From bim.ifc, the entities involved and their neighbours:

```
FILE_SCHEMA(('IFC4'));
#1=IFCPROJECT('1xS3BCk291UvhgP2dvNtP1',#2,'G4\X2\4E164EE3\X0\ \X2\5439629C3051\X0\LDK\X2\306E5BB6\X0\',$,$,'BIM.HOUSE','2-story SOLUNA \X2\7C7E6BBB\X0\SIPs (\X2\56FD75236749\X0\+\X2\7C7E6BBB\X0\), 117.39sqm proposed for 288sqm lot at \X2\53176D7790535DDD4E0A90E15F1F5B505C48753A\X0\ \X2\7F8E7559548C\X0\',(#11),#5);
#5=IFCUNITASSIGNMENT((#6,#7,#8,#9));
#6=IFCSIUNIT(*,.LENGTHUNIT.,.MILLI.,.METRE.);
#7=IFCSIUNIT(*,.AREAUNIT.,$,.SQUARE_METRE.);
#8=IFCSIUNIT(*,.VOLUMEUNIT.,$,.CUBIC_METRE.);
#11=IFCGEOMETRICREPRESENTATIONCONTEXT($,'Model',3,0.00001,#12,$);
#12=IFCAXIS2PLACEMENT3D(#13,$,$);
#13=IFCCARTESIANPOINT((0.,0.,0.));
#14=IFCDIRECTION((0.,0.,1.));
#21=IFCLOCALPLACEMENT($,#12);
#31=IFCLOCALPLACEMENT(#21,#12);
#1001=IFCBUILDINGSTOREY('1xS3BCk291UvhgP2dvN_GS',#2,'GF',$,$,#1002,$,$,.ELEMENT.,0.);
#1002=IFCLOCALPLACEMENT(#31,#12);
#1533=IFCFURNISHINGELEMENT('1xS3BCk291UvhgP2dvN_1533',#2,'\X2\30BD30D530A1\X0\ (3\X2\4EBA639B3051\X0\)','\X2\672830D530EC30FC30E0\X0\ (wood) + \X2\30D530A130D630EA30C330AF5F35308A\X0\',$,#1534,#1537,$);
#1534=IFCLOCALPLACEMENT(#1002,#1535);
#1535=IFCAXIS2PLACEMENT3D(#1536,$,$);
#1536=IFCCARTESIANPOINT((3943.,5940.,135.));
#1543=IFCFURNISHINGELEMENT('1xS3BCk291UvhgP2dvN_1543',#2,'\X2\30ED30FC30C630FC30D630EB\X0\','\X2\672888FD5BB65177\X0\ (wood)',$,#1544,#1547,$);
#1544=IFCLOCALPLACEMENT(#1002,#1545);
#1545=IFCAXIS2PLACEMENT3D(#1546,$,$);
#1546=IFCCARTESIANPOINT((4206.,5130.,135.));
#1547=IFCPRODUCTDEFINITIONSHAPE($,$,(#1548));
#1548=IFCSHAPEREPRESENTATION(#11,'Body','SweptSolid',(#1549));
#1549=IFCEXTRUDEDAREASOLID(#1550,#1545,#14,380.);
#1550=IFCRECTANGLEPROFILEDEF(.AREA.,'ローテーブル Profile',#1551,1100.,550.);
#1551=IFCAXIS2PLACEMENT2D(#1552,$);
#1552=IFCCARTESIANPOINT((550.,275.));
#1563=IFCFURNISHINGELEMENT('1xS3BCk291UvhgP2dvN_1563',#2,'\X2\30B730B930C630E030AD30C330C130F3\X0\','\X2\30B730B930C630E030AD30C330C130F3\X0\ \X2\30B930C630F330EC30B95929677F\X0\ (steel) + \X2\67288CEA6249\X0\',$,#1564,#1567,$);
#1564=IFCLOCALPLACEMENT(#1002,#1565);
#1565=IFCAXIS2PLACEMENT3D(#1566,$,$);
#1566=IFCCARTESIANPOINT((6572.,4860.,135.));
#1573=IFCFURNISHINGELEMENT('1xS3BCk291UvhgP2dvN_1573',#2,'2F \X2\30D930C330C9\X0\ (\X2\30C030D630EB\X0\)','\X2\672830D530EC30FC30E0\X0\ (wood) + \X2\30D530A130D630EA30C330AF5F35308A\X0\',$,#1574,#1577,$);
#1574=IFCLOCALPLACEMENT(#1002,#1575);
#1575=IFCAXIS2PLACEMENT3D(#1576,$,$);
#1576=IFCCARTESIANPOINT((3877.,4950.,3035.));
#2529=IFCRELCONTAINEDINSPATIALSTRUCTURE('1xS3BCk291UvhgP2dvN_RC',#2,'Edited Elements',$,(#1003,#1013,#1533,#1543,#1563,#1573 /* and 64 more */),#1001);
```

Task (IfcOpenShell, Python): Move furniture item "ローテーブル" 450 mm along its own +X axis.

```python
import ifcopenshell
import ifcopenshell.api.geometry
import ifcopenshell.util.placement

model = ifcopenshell.open("bim.ifc")

item = model.by_id(1543)
matrix = ifcopenshell.util.placement.get_local_placement(item.ObjectPlacement)
matrix[:3, 3] += matrix[:3, 0] * 450.0
ifcopenshell.api.geometry.edit_object_placement(model, product=item, matrix=matrix, is_si=False)

print(ifcopenshell.util.placement.get_local_placement(item.ObjectPlacement).round(3) + 0.0)

model.write("bim_edited.ifc")
```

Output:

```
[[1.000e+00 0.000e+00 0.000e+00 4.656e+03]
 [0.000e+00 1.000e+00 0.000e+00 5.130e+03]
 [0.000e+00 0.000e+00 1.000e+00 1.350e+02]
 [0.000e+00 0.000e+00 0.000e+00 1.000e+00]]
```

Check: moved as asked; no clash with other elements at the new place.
